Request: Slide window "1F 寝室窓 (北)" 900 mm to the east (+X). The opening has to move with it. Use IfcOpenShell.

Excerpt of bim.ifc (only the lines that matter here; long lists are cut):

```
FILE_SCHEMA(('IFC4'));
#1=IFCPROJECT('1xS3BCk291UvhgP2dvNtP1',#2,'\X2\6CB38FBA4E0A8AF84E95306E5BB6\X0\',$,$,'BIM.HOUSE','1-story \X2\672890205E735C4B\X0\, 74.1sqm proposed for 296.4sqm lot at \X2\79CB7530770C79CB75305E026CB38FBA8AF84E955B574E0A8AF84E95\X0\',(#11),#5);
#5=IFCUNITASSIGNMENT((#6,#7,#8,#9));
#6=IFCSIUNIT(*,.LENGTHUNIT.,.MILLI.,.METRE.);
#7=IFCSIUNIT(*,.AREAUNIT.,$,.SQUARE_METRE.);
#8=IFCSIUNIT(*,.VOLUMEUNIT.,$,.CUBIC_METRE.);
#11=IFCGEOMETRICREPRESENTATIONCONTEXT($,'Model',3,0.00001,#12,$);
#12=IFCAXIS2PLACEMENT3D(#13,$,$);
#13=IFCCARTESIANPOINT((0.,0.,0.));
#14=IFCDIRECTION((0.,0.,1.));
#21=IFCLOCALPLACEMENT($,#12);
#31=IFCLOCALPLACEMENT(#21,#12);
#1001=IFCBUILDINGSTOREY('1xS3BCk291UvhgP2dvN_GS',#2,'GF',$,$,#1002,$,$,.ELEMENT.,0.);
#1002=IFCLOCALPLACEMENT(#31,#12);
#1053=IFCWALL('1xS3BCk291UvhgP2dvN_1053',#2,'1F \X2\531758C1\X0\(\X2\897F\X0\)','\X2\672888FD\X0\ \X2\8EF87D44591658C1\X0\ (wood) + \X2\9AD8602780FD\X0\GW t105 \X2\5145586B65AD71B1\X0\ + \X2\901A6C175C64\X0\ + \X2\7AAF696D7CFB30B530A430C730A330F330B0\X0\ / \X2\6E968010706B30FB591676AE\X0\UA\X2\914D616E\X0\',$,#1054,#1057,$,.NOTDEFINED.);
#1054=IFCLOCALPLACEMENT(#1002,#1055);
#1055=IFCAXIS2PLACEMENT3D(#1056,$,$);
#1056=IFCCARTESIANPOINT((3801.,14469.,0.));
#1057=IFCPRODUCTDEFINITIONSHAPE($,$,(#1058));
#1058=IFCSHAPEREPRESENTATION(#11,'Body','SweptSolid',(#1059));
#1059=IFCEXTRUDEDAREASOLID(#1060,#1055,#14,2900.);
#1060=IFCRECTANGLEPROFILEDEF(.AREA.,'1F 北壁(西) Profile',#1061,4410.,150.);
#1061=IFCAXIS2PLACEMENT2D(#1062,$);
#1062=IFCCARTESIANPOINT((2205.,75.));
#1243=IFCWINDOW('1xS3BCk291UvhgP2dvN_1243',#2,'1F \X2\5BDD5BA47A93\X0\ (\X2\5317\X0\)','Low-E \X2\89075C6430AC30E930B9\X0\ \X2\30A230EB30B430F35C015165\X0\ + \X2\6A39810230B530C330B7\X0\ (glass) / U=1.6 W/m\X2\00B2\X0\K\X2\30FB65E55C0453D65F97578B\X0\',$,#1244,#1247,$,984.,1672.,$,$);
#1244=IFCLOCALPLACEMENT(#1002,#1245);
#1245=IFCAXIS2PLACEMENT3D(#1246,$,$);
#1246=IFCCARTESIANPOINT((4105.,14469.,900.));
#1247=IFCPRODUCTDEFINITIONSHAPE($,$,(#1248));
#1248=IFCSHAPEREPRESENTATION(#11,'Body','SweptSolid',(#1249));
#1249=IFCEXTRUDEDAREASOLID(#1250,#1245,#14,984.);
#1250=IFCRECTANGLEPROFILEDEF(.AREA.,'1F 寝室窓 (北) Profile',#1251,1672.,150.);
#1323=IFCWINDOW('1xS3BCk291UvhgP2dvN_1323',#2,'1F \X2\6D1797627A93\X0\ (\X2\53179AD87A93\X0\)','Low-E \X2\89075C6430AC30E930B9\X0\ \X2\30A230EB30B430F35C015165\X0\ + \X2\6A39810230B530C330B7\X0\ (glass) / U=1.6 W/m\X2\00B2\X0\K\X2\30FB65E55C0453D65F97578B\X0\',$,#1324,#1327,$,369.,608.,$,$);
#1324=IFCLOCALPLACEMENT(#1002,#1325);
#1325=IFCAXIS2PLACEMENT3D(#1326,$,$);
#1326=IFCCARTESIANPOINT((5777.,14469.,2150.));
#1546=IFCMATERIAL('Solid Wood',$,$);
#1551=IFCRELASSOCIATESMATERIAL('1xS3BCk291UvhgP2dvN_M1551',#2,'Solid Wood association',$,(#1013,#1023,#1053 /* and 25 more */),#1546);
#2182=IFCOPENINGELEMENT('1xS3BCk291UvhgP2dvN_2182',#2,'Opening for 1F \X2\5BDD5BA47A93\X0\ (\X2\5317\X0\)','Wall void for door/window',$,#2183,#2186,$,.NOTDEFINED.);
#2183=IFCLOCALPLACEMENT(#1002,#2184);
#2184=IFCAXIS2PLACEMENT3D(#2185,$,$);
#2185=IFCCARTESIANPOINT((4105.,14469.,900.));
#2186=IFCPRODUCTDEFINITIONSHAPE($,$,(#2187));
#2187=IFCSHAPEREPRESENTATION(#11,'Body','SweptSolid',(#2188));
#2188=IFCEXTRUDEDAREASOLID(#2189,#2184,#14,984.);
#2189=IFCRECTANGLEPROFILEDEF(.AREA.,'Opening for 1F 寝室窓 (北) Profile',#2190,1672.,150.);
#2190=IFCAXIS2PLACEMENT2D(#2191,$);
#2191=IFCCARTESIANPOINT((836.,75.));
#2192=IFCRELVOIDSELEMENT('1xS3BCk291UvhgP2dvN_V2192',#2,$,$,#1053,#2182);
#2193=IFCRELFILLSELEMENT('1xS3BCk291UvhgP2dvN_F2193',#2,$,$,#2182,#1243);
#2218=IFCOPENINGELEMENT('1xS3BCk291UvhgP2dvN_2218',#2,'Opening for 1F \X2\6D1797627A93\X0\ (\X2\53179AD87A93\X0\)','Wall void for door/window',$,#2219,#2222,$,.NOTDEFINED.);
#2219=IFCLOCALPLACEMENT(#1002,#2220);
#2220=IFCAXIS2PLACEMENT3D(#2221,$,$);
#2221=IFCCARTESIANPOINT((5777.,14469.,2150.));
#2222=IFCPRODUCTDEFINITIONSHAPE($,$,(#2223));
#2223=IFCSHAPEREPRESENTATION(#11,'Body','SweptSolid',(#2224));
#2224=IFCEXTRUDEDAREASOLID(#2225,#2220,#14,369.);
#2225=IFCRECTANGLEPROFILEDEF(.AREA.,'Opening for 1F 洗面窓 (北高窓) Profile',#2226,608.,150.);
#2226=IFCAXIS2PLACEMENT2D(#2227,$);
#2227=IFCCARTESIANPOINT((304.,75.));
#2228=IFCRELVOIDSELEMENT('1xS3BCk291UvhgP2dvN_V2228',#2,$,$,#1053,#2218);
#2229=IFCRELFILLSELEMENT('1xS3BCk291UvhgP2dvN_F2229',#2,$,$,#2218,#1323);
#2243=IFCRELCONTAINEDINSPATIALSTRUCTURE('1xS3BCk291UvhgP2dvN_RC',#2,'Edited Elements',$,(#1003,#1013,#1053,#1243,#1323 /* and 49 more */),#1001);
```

```python
import ifcopenshell
import ifcopenshell.api.geometry
import ifcopenshell.util.placement
import ifcopenshell.util.unit

model = ifcopenshell.open("bim.ifc")
unit_scale = ifcopenshell.util.unit.calculate_unit_scale(model)

window = model.by_id(1243)
opening = window.FillsVoids[0].RelatingOpeningElement
wall = opening.VoidsElements[0].RelatingBuildingElement

wall_matrix = ifcopenshell.util.placement.get_local_placement(wall.ObjectPlacement)
shift = wall_matrix[:3, 0] * 0.9 / unit_scale
before = ifcopenshell.util.placement.get_local_placement(window.ObjectPlacement)[:3, 3].copy()

# The window is not placed relative to its opening, so move both.
for product in (opening, window):
    matrix = ifcopenshell.util.placement.get_local_placement(product.ObjectPlacement)
    matrix[:3, 3] += shift
    ifcopenshell.api.geometry.edit_object_placement(model, product=product, matrix=matrix, is_si=False)

after = ifcopenshell.util.placement.get_local_placement(window.ObjectPlacement)[:3, 3]
print("window moved by", (after - before).round(3) + 0.0)

model.write("bim_edited.ifc")
```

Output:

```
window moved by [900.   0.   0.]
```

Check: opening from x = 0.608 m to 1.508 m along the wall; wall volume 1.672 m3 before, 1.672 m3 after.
